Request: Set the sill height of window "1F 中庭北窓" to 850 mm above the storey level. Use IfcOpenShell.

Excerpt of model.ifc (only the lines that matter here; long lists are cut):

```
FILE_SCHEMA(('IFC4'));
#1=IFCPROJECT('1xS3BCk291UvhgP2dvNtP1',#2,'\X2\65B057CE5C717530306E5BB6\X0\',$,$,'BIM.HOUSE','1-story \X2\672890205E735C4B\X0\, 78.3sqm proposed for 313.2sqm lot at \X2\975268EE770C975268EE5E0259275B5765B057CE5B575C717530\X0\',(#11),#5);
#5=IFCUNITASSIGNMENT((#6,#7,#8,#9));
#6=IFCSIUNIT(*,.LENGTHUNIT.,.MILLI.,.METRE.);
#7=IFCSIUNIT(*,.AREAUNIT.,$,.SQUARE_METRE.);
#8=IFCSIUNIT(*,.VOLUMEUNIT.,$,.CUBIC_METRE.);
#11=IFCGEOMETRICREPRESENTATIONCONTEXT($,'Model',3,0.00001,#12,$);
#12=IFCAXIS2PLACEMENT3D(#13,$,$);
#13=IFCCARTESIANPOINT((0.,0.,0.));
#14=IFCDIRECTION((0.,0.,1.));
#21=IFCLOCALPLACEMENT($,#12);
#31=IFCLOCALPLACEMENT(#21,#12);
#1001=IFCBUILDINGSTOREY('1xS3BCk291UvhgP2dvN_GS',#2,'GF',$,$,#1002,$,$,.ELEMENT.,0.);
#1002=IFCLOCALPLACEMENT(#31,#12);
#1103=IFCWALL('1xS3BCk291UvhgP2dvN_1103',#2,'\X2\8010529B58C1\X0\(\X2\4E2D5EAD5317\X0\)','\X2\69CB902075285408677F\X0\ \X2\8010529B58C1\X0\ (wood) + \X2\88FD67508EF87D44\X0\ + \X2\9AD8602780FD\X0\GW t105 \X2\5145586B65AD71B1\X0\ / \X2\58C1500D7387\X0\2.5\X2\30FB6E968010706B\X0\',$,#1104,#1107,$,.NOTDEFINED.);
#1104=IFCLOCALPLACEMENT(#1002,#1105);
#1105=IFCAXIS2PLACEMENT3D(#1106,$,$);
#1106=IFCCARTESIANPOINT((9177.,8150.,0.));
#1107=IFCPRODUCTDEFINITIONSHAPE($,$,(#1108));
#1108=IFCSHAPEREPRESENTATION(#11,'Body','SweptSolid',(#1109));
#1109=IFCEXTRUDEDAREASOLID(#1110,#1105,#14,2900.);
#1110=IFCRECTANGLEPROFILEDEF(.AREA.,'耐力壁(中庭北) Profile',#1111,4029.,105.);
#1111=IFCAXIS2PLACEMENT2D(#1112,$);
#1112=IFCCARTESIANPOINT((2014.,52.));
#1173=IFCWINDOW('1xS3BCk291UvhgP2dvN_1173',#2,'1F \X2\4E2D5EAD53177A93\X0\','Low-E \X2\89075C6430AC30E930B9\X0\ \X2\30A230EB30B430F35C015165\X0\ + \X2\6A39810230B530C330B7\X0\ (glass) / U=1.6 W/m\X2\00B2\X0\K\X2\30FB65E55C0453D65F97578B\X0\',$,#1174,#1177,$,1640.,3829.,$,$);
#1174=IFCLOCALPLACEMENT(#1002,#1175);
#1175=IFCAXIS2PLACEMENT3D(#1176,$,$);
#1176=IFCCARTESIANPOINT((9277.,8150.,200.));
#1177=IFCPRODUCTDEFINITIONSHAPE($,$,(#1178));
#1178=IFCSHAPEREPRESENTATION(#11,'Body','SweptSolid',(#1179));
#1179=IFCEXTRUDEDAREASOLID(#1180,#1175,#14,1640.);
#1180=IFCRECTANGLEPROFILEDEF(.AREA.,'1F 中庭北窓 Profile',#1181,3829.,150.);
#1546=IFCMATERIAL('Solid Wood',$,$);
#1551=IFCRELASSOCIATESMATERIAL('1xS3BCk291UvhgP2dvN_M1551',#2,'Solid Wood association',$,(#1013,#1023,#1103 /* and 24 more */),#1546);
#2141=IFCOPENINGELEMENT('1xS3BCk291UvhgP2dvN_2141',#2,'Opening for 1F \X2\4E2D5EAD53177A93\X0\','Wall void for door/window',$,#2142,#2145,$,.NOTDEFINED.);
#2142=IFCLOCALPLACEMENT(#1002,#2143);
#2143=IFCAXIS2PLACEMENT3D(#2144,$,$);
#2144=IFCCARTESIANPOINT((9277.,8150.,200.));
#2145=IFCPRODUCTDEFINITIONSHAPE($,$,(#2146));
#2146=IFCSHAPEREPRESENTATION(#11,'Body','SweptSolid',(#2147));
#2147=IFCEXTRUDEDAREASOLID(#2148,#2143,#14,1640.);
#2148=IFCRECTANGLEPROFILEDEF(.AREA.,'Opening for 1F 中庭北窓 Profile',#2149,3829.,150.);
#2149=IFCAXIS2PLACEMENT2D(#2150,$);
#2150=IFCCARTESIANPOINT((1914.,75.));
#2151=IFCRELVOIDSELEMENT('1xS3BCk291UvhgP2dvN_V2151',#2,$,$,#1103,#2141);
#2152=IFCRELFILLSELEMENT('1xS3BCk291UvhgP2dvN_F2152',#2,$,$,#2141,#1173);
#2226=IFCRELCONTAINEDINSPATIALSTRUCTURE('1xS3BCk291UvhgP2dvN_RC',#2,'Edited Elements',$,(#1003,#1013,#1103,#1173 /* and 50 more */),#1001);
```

```python
import numpy as np
import ifcopenshell
import ifcopenshell.api.geometry
import ifcopenshell.geom
import ifcopenshell.util.element
import ifcopenshell.util.placement
import ifcopenshell.util.shape
import ifcopenshell.util.unit

model = ifcopenshell.open("model.ifc")
unit_scale = ifcopenshell.util.unit.calculate_unit_scale(model)

window = model.by_id(1173)
opening = window.FillsVoids[0].RelatingOpeningElement
storey = ifcopenshell.util.element.get_container(window, ifc_class="IfcBuildingStorey")
level = ifcopenshell.util.placement.get_local_placement(storey.ObjectPlacement)[2, 3]

# The opening's origin need not be at the sill, so measure its lowest point.
shape = ifcopenshell.geom.create_shape(ifcopenshell.geom.settings(), opening)
bottom = ifcopenshell.util.shape.get_shape_bottom_elevation(shape, shape.geometry) / unit_scale
dz = level + 0.85 / unit_scale - bottom

shift = np.array([0.0, 0.0, dz])
# The window is not placed relative to its opening, so move both.
for product in (opening, window):
    matrix = ifcopenshell.util.placement.get_local_placement(product.ObjectPlacement)
    matrix[:3, 3] += shift
    ifcopenshell.api.geometry.edit_object_placement(model, product=product, matrix=matrix, is_si=False)

print(f"moved by {dz * unit_scale:+.3f} m")

model.write("model_v2.ifc")
```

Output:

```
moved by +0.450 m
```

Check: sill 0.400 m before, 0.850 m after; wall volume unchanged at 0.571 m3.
